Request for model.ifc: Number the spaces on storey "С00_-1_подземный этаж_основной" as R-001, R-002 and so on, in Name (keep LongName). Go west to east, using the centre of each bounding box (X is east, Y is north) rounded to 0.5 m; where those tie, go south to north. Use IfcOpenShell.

First a look at what the model holds.

```python
import ifcopenshell
import ifcopenshell.util.element
import ifcopenshell.util.placement

model = ifcopenshell.open("model.ifc")
print(model.schema)
storey = next(s for s in model.by_type("IfcBuildingStorey") if s.Name == "С00_-1_подземный этаж_основной")
spaces = [e for e in ifcopenshell.util.element.get_decomposition(storey) if e.is_a("IfcSpace")]
for e in sorted(spaces, key=lambda e: e.id()):
    origin = ifcopenshell.util.placement.get_local_placement(e.ObjectPlacement)[:3, 3]
    print(e.id(), e.Name, e.LongName, origin.round(2) + 0.0, sep=" | ")
```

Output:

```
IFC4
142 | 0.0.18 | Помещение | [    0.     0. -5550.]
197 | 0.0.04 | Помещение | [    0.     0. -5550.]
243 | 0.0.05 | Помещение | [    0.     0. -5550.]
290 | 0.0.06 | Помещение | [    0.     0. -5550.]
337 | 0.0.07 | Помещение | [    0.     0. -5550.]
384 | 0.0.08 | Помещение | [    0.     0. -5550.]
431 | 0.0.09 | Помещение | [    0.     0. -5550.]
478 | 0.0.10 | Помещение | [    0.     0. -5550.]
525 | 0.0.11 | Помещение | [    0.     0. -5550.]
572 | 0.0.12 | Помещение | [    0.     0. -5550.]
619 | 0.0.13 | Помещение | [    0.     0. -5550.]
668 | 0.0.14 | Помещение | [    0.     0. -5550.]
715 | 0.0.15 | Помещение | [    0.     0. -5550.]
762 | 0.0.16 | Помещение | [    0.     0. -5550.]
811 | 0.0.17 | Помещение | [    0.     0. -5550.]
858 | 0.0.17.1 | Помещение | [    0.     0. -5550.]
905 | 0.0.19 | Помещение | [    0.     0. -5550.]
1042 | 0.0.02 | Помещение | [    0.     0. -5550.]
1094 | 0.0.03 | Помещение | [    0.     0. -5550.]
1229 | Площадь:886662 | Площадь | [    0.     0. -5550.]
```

```python
import ifcopenshell
import ifcopenshell.geom
import ifcopenshell.util.element
import ifcopenshell.util.shape

model = ifcopenshell.open("model.ifc")
settings = ifcopenshell.geom.settings()
settings.set("use-world-coords", True)


def centre(element):
    shape = ifcopenshell.geom.create_shape(settings, element)
    return ifcopenshell.util.shape.get_bbox_centroid(shape.geometry)


storey = next(s for s in model.by_type("IfcBuildingStorey") if s.Name == "С00_-1_подземный этаж_основной")
spaces = [e for e in ifcopenshell.util.element.get_decomposition(storey) if e.is_a("IfcSpace")]

# Insertion points can sit at a corner or the storey origin, so sort by the geometry (in metres).
centres = {e: centre(e) for e in spaces}
spaces.sort(key=lambda e: (round(centres[e][0] / 0.5), centres[e][1]))

for i, e in enumerate(spaces, start=1):
    number = f"R-0{i:02d}"
    e.Name = number
    print(e.id(), number)

model.write("model-out.ifc")
```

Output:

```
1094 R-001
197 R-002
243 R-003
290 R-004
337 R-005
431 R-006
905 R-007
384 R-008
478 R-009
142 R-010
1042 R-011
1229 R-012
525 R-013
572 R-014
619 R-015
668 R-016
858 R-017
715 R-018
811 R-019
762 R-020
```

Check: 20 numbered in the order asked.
